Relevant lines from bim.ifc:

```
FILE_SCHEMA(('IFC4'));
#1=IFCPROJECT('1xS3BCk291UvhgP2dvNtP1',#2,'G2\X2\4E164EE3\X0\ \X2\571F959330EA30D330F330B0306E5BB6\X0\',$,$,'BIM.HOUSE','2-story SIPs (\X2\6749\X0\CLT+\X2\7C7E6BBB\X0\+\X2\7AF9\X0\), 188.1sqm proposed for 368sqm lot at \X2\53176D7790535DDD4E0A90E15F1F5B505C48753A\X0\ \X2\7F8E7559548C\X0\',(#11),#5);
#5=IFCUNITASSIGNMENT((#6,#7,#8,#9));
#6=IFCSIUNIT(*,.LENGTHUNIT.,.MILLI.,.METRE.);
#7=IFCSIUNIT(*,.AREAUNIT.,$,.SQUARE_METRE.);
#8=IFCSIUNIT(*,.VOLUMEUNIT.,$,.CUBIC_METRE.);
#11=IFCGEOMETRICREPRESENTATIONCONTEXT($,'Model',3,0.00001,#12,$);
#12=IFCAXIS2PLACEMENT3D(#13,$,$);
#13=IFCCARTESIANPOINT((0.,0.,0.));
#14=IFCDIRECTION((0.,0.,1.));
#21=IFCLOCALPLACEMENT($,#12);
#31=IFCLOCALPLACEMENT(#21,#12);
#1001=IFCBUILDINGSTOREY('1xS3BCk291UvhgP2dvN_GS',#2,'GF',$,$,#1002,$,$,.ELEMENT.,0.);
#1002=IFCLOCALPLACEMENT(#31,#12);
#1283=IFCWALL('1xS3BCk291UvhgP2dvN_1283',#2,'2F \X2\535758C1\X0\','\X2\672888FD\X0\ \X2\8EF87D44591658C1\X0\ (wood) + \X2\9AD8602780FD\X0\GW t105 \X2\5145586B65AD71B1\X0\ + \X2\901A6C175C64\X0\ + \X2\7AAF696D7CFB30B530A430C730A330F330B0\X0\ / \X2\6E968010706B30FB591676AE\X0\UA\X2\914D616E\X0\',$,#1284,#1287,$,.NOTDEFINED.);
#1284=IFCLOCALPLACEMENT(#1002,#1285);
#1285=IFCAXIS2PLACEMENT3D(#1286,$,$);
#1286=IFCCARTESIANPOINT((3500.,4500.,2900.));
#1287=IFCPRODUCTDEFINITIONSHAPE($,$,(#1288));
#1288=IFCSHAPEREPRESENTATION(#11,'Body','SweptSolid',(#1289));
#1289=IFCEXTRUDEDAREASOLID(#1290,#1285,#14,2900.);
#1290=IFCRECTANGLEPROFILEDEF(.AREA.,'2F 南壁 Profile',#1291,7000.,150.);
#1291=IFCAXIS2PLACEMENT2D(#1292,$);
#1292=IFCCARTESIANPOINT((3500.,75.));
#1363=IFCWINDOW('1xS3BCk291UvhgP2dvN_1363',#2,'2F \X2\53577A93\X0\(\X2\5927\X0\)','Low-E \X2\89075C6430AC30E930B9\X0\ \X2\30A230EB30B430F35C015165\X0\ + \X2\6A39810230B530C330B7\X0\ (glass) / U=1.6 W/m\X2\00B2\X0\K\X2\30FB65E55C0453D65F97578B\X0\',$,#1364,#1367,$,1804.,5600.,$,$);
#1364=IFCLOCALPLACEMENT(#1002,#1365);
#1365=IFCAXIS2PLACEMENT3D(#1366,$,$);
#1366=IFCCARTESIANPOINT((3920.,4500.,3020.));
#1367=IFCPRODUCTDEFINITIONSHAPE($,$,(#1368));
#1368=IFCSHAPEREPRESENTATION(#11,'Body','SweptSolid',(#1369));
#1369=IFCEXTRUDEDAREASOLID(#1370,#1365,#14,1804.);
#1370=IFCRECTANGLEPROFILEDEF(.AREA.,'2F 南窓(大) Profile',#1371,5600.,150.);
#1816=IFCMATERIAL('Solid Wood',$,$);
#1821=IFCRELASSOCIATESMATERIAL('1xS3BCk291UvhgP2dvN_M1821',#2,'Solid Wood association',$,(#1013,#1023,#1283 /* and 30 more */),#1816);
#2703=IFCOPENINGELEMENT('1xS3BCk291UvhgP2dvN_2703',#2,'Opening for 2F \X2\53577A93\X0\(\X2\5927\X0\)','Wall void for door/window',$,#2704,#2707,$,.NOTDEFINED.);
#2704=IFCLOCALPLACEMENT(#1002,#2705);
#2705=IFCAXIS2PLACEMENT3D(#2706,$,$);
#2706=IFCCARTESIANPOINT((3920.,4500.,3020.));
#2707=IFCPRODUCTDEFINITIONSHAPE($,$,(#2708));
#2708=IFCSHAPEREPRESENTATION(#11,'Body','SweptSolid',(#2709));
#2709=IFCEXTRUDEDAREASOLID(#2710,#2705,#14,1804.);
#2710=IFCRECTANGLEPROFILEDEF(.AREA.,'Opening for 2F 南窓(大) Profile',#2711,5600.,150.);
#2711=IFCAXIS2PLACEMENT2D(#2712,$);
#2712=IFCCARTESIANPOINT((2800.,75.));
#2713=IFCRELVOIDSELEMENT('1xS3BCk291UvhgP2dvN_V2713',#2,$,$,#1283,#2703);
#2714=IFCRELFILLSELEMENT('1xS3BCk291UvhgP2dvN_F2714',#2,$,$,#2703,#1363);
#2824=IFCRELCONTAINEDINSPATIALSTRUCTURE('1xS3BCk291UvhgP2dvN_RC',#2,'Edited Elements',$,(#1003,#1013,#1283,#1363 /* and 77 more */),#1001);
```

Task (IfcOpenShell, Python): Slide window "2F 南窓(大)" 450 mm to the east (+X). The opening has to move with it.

```python
import ifcopenshell
import ifcopenshell.api.geometry
import ifcopenshell.util.placement
import ifcopenshell.util.unit

model = ifcopenshell.open("bim.ifc")
unit_scale = ifcopenshell.util.unit.calculate_unit_scale(model)

window = model.by_guid("1xS3BCk291UvhgP2dvN_1363")
opening = window.FillsVoids[0].RelatingOpeningElement
wall = opening.VoidsElements[0].RelatingBuildingElement

wall_matrix = ifcopenshell.util.placement.get_local_placement(wall.ObjectPlacement)
shift = wall_matrix[:3, 0] * 0.45 / unit_scale
before = ifcopenshell.util.placement.get_local_placement(window.ObjectPlacement)[:3, 3].copy()

# The window is not placed relative to its opening, so move both.
for product in (opening, window):
    matrix = ifcopenshell.util.placement.get_local_placement(product.ObjectPlacement)
    matrix[:3, 3] += shift
    ifcopenshell.api.geometry.edit_object_placement(model, product=product, matrix=matrix, is_si=False)

after = ifcopenshell.util.placement.get_local_placement(window.ObjectPlacement)[:3, 3]
print("window moved by", (after - before).round(3) + 0.0)

model.write("bim_rev.ifc")
```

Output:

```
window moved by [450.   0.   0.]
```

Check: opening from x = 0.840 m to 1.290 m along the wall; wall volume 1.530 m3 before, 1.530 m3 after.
